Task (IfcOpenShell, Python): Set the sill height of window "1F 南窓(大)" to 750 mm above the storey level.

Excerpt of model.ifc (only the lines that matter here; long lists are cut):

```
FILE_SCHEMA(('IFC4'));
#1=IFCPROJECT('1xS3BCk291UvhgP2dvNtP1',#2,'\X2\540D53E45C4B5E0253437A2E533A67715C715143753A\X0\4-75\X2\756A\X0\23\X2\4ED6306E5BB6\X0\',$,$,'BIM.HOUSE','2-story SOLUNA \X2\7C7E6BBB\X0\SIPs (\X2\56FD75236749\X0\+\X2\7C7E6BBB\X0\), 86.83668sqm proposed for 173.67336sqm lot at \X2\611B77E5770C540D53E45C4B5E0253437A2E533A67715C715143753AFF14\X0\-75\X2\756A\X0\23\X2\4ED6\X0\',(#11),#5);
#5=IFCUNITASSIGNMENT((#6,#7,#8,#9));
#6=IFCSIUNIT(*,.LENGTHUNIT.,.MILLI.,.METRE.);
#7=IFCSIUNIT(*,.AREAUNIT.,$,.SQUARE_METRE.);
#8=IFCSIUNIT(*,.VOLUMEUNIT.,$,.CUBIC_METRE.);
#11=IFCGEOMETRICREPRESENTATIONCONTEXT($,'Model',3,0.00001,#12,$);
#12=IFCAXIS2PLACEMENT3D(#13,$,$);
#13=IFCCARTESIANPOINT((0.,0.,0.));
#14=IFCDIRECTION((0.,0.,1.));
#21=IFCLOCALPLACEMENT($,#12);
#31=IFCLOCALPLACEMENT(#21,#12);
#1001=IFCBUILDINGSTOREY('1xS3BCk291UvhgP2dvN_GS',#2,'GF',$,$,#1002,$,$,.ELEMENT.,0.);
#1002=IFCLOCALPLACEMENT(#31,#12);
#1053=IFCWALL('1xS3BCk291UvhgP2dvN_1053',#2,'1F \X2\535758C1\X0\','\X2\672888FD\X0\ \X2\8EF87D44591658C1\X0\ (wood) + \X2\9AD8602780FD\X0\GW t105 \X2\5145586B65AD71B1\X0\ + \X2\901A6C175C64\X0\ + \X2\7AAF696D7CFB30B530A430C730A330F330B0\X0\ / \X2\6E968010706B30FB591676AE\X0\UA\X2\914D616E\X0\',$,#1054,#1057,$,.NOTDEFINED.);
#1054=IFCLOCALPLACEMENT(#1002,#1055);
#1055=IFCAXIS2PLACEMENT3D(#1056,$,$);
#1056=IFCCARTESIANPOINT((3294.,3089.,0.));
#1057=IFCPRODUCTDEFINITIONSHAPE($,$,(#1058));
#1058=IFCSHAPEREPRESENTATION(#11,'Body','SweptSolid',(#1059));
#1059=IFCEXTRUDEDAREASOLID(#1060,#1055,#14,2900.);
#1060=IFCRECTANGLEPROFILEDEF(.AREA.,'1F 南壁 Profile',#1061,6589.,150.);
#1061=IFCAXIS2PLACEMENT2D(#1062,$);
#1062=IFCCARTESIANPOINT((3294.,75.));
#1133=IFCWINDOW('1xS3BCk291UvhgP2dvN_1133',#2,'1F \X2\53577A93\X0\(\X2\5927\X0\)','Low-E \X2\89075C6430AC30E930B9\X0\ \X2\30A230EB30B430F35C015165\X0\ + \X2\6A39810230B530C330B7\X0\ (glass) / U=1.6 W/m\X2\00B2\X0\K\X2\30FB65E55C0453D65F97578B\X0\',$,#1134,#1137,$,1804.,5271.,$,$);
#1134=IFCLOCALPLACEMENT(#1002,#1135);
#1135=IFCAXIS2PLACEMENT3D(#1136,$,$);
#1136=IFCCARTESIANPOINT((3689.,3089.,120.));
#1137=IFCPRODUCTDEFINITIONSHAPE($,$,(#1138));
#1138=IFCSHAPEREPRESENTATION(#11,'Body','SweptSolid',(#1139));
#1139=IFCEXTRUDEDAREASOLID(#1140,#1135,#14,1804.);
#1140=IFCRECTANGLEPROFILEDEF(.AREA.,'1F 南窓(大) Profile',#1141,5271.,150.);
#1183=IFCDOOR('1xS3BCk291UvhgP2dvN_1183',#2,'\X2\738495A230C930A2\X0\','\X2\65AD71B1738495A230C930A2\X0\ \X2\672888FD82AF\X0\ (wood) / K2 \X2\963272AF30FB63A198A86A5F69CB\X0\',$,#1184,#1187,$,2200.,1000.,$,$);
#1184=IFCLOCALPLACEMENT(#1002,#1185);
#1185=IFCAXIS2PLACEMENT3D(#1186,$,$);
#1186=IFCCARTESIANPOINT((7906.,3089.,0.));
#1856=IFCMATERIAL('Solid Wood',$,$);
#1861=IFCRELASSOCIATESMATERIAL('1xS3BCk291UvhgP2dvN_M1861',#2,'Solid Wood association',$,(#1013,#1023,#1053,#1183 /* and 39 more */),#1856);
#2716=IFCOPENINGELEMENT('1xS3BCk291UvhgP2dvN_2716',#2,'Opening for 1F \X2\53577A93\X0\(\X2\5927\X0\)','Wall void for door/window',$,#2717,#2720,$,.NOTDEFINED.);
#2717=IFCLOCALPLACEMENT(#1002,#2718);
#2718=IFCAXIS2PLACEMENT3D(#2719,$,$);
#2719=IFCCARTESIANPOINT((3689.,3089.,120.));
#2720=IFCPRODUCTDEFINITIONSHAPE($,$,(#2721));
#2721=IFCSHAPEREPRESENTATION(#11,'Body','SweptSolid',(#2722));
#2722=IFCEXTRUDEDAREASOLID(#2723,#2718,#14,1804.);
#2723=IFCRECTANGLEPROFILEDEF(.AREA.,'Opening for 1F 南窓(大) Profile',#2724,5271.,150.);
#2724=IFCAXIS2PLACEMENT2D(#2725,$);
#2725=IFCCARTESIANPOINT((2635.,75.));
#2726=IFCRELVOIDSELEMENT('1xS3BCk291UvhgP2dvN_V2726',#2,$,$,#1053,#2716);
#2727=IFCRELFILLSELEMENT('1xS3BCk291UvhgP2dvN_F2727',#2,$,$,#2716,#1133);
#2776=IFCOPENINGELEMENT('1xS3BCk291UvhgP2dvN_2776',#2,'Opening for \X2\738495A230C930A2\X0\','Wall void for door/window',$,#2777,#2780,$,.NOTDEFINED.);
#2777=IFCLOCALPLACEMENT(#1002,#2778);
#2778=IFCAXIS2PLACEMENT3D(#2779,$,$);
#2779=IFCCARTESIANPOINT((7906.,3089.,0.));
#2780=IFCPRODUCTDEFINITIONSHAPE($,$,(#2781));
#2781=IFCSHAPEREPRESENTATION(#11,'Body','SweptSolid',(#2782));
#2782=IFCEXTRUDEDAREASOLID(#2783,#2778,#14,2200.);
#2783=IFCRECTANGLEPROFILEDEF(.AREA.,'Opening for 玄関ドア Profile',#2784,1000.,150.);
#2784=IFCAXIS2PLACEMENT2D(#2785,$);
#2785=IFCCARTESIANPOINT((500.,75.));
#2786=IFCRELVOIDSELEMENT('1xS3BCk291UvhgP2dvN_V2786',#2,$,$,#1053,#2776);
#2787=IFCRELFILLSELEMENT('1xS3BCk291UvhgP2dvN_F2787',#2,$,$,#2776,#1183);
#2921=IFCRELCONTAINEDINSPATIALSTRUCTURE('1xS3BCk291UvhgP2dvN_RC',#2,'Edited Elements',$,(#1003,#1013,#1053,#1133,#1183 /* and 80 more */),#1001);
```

```python
import numpy as np
import ifcopenshell
import ifcopenshell.api.geometry
import ifcopenshell.geom
import ifcopenshell.util.element
import ifcopenshell.util.placement
import ifcopenshell.util.shape
import ifcopenshell.util.unit

model = ifcopenshell.open("model.ifc")
unit_scale = ifcopenshell.util.unit.calculate_unit_scale(model)

window = model.by_guid("1xS3BCk291UvhgP2dvN_1133")
opening = window.FillsVoids[0].RelatingOpeningElement
storey = ifcopenshell.util.element.get_container(window, ifc_class="IfcBuildingStorey")
level = ifcopenshell.util.placement.get_local_placement(storey.ObjectPlacement)[2, 3]

# The opening's origin need not be at the sill, so measure its lowest point.
shape = ifcopenshell.geom.create_shape(ifcopenshell.geom.settings(), opening)
bottom = ifcopenshell.util.shape.get_shape_bottom_elevation(shape, shape.geometry) / unit_scale
dz = level + 0.75 / unit_scale - bottom

shift = np.array([0.0, 0.0, dz])
# The window is not placed relative to its opening, so move both.
for product in (opening, window):
    matrix = ifcopenshell.util.placement.get_local_placement(product.ObjectPlacement)
    matrix[:3, 3] += shift
    ifcopenshell.api.geometry.edit_object_placement(model, product=product, matrix=matrix, is_si=False)

print(f"moved by {dz * unit_scale:+.3f} m")

model.write("model_v2.ifc")
```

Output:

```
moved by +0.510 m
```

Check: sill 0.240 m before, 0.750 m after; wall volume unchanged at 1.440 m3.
